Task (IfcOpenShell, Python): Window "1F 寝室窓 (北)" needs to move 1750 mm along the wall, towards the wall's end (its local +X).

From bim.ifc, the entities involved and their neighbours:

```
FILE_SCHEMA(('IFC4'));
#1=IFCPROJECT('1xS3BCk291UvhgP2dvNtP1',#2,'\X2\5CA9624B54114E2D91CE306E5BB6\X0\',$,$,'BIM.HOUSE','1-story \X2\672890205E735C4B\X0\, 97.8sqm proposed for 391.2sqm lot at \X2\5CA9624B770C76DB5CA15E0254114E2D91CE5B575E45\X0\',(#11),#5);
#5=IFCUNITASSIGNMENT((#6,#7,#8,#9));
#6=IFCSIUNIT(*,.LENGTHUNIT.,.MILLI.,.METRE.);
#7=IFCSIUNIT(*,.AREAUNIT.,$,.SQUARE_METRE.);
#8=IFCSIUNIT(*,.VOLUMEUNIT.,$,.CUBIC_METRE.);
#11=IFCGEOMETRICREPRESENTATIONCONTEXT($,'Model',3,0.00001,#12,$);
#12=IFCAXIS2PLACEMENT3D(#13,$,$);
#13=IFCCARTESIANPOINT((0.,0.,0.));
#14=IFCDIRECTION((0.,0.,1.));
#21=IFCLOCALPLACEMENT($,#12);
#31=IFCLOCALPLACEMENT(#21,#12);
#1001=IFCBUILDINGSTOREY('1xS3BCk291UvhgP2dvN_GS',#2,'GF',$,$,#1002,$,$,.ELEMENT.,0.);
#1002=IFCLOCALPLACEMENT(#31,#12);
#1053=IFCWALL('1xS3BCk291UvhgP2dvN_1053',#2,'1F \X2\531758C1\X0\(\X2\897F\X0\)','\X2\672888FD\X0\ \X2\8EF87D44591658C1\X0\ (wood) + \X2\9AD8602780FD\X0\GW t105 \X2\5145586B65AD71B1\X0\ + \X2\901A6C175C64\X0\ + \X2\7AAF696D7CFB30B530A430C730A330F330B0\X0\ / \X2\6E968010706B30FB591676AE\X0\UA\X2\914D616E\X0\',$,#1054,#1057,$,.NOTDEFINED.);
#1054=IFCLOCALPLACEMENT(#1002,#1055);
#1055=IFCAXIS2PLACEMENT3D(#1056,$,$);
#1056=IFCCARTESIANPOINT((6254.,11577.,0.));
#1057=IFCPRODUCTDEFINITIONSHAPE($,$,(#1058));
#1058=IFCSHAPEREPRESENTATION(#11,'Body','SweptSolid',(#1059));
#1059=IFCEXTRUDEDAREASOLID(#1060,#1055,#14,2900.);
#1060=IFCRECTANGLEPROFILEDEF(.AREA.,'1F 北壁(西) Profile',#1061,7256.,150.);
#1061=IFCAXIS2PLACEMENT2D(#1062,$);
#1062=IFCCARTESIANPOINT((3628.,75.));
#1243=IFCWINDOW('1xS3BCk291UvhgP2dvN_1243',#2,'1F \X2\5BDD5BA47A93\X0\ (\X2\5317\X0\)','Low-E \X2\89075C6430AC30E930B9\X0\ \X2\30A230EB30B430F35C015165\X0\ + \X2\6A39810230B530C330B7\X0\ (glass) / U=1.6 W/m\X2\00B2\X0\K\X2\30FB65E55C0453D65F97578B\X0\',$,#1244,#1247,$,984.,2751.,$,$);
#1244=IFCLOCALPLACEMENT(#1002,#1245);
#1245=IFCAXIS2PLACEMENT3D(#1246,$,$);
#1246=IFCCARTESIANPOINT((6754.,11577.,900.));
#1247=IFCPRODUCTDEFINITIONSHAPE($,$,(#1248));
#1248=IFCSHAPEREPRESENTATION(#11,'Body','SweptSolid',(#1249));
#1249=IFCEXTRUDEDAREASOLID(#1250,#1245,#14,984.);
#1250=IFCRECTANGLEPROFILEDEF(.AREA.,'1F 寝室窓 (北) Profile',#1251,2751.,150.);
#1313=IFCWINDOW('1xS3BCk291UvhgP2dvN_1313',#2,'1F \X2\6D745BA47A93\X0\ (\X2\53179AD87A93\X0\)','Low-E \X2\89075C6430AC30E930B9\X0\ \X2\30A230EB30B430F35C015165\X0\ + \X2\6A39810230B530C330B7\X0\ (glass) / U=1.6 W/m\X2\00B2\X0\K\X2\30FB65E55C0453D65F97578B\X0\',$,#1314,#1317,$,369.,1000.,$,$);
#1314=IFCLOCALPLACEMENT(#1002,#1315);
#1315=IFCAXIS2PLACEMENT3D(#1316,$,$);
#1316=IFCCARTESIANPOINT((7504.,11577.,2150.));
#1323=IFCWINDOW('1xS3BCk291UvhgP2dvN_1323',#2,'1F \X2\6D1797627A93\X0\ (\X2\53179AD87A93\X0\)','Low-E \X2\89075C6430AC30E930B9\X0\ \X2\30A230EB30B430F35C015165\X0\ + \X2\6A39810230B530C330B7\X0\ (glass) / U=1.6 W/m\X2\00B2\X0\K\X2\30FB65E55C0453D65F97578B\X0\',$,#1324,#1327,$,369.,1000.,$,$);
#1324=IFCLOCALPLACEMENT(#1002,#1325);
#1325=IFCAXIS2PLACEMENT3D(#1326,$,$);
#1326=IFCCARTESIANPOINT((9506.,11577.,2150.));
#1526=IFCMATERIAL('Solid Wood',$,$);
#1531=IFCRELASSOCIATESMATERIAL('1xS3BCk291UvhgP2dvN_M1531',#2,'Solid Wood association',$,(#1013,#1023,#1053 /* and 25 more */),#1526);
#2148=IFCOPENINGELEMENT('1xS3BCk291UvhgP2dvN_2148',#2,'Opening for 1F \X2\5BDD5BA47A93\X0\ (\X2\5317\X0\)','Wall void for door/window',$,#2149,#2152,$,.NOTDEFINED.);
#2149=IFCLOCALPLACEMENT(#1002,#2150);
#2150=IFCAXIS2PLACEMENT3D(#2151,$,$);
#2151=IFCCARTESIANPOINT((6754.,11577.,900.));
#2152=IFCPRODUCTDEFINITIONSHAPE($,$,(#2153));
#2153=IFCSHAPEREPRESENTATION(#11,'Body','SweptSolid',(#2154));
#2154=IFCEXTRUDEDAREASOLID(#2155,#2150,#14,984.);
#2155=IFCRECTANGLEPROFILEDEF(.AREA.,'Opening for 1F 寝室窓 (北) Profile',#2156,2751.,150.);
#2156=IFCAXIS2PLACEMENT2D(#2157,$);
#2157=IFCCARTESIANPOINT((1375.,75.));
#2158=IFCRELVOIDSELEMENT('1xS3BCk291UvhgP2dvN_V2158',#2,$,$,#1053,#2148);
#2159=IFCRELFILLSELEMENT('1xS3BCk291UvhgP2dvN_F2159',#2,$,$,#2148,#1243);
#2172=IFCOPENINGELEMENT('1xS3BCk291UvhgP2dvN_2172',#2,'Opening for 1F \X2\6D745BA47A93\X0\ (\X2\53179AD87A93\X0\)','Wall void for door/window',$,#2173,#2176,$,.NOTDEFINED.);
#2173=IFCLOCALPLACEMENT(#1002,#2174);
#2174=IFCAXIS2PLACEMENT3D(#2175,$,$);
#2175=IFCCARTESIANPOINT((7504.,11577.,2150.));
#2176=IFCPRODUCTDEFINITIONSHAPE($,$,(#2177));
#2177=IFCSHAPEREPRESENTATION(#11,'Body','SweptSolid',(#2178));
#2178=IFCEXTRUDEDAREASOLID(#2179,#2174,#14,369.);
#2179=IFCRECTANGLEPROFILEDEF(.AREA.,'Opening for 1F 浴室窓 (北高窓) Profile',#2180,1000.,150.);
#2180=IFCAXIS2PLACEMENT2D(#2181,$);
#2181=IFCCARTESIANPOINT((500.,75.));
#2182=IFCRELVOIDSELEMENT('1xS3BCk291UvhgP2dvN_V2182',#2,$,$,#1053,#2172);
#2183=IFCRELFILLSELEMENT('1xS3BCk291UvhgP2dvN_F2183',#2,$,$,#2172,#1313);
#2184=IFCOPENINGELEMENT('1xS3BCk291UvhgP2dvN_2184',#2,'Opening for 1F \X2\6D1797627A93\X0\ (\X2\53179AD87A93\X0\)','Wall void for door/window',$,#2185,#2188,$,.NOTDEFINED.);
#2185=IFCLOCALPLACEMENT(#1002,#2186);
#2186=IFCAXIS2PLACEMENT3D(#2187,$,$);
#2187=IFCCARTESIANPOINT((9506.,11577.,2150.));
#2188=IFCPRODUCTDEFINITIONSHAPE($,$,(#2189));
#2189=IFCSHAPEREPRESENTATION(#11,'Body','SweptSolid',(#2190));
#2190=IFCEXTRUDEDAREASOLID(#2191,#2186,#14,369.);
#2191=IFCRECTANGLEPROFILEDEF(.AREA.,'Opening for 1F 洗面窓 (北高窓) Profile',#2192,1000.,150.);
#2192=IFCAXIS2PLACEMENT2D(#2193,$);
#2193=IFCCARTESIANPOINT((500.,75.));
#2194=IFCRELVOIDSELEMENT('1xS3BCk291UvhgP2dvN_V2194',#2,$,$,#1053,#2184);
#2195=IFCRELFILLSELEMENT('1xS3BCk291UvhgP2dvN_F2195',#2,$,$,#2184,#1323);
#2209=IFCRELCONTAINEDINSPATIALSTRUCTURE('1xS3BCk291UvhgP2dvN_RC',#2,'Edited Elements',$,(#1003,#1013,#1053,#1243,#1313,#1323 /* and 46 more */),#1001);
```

```python
import ifcopenshell
import ifcopenshell.api.geometry
import ifcopenshell.util.placement
import ifcopenshell.util.unit

model = ifcopenshell.open("bim.ifc")
unit_scale = ifcopenshell.util.unit.calculate_unit_scale(model)

window = model.by_id(1243)
opening = window.FillsVoids[0].RelatingOpeningElement
wall = opening.VoidsElements[0].RelatingBuildingElement

wall_matrix = ifcopenshell.util.placement.get_local_placement(wall.ObjectPlacement)
shift = wall_matrix[:3, 0] * 1.75 / unit_scale
before = ifcopenshell.util.placement.get_local_placement(window.ObjectPlacement)[:3, 3].copy()

# The window is not placed relative to its opening, so move both.
for product in (opening, window):
    matrix = ifcopenshell.util.placement.get_local_placement(product.ObjectPlacement)
    matrix[:3, 3] += shift
    ifcopenshell.api.geometry.edit_object_placement(model, product=product, matrix=matrix, is_si=False)

after = ifcopenshell.util.placement.get_local_placement(window.ObjectPlacement)[:3, 3]
print("window moved by", (after - before).round(3) + 0.0)

model.write("bim-out.ifc")
```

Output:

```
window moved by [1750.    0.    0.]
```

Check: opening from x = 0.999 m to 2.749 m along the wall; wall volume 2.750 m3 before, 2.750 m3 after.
